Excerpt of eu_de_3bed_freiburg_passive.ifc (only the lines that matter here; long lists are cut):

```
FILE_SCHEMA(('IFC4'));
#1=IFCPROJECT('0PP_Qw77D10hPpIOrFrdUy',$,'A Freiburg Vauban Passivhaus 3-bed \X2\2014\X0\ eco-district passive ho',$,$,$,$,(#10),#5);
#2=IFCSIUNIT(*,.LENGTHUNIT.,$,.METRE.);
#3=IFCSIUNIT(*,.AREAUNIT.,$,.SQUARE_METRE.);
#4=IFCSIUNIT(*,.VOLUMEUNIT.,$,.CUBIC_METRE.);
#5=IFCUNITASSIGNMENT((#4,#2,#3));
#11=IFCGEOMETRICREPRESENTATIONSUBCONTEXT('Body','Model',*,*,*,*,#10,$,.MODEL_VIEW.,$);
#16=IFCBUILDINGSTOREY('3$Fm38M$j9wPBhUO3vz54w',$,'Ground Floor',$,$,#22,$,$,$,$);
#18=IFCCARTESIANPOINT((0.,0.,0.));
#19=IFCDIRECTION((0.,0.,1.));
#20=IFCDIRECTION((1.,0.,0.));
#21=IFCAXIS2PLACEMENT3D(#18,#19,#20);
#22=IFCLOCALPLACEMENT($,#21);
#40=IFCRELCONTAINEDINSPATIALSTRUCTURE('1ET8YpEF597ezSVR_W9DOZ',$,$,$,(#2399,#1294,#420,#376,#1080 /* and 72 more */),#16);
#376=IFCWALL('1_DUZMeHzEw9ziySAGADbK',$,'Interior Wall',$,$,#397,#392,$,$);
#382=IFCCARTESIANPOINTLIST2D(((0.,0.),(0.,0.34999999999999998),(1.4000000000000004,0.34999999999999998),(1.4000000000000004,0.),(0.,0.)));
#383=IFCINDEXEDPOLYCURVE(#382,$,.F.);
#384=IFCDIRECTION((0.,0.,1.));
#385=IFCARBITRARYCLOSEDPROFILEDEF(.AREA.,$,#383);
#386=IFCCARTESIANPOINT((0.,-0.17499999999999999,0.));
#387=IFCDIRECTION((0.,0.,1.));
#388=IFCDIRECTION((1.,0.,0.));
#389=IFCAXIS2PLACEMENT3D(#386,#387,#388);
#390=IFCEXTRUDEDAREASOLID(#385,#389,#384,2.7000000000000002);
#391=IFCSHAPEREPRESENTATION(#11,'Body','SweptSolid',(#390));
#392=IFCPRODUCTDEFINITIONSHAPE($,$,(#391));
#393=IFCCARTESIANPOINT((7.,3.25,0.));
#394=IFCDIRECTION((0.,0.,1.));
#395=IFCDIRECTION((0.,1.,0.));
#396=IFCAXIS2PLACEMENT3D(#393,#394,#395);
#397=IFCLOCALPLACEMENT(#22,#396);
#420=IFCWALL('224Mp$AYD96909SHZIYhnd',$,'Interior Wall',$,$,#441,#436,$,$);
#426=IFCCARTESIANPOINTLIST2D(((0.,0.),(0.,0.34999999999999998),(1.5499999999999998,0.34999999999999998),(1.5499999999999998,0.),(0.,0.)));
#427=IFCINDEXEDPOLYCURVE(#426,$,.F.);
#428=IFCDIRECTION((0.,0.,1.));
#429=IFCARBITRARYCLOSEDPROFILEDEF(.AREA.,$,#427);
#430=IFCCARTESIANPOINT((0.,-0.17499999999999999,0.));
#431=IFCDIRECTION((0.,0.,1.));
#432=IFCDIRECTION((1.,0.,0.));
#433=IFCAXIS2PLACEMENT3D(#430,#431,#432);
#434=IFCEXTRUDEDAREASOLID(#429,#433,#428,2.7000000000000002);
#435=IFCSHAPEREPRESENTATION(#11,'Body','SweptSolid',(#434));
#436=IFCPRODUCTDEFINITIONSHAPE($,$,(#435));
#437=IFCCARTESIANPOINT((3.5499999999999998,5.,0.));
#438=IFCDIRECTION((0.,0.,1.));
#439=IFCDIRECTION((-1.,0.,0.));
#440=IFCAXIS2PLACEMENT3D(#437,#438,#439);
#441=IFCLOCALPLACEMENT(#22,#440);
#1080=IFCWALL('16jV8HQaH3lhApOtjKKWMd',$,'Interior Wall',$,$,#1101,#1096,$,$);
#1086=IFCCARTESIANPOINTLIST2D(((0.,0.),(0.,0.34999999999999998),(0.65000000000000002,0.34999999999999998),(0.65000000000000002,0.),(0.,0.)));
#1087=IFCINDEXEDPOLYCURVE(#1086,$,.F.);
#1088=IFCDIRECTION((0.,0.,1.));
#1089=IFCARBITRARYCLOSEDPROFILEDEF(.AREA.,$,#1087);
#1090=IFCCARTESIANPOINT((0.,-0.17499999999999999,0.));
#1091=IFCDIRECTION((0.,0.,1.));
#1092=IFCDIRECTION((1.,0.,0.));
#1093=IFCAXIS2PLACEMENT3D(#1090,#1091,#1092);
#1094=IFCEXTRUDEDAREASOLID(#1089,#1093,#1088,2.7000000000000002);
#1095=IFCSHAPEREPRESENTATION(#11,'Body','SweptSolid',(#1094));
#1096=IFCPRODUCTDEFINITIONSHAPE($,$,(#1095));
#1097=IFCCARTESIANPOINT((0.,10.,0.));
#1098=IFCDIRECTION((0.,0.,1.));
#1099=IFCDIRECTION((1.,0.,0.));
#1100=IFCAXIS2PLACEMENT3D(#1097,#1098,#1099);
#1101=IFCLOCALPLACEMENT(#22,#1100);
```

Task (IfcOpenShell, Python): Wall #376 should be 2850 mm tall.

```python
import ifcopenshell
import ifcopenshell.geom
import ifcopenshell.util.representation
import ifcopenshell.util.shape

model = ifcopenshell.open("eu_de_3bed_freiburg_passive.ifc")
settings = ifcopenshell.geom.settings()


def volume(element):
    """Net volume in cubic metres, openings subtracted."""
    shape = ifcopenshell.geom.create_shape(settings, element)
    return ifcopenshell.util.shape.get_volume(shape.geometry)


wall = model.by_id(376)
before = volume(wall)

body = ifcopenshell.util.representation.get_representation(wall, "Model", "Body")
solid = body.Items[0]
old_height = solid.Depth
solid.Depth = 2.85
after = volume(wall)

print(f"height {old_height:g} -> {solid.Depth:g}, volume {before:.3f} -> {after:.3f} m3")

model.write("eu_de_3bed_freiburg_passive_rev.ifc")
```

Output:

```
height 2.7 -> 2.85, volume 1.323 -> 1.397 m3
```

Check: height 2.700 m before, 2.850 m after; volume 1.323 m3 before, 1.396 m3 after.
